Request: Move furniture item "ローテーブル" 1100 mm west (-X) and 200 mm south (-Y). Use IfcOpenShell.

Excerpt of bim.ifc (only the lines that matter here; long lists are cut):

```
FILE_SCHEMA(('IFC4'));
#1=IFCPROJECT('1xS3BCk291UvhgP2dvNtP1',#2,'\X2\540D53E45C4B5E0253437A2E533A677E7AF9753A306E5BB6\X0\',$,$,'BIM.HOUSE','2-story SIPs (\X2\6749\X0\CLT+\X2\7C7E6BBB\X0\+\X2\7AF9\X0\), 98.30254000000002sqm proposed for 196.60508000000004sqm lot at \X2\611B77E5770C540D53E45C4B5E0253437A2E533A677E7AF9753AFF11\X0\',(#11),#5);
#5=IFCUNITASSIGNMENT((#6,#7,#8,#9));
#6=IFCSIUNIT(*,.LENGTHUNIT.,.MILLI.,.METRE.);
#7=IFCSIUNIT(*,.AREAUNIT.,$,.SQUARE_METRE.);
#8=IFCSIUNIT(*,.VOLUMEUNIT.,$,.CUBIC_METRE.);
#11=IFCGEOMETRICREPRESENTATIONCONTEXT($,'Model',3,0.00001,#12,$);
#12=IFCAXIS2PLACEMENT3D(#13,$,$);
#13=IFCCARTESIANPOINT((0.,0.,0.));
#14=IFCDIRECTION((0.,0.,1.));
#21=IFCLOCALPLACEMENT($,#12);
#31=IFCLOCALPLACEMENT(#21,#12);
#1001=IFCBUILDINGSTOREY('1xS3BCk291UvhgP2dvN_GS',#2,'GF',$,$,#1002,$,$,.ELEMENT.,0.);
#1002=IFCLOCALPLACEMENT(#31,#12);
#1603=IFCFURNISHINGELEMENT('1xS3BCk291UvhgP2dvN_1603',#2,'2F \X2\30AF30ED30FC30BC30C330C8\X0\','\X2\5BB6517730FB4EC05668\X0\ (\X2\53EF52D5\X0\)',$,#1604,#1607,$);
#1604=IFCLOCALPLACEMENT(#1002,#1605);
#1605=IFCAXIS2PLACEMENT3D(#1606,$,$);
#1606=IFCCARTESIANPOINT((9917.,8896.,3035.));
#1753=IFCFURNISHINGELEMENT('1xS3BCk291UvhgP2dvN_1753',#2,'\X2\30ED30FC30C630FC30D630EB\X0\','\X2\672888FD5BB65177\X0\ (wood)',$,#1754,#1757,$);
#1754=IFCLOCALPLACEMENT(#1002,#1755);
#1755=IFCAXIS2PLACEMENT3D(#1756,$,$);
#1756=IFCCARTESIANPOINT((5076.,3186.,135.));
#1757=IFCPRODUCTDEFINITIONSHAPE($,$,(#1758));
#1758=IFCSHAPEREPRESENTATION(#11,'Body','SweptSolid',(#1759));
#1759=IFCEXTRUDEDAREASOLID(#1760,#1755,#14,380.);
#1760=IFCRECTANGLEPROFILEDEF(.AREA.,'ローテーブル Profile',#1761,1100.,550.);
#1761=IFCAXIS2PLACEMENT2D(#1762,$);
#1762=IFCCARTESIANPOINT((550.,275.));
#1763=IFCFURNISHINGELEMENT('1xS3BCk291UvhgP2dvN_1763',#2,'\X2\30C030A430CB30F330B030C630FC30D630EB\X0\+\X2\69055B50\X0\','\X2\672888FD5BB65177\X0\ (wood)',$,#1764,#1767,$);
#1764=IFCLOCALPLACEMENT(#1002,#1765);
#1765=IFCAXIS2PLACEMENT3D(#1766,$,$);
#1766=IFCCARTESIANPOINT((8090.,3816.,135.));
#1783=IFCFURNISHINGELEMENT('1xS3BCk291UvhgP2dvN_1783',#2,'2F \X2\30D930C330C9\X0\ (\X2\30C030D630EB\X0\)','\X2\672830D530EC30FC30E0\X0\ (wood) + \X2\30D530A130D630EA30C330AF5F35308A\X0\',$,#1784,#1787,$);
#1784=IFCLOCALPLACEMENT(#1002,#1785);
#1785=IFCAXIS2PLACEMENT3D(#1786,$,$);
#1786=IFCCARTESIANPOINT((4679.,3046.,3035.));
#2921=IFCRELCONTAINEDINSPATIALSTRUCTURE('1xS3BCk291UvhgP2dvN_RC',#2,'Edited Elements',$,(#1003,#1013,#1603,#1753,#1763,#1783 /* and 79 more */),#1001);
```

```python
import ifcopenshell
import ifcopenshell.api.geometry
import ifcopenshell.util.placement
import ifcopenshell.util.unit

model = ifcopenshell.open("bim.ifc")
unit_scale = ifcopenshell.util.unit.calculate_unit_scale(model)

item = model.by_guid("1xS3BCk291UvhgP2dvN_1753")
matrix = ifcopenshell.util.placement.get_local_placement(item.ObjectPlacement)
matrix[0, 3] -= 1.1 / unit_scale
matrix[1, 3] -= 0.2 / unit_scale
ifcopenshell.api.geometry.edit_object_placement(model, product=item, matrix=matrix, is_si=False)

print(ifcopenshell.util.placement.get_local_placement(item.ObjectPlacement).round(3) + 0.0)

model.write("bim_v2.ifc")
```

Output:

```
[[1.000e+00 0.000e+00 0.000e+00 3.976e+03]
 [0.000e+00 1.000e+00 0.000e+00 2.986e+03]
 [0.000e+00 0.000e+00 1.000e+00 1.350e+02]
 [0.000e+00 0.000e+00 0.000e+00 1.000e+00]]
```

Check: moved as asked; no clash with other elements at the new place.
